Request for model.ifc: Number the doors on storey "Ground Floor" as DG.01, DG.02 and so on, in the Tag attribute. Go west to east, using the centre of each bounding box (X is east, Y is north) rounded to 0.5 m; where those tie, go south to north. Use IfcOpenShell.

First a look at what the model holds.

```python
import ifcopenshell
import ifcopenshell.util.element
import ifcopenshell.util.placement

model = ifcopenshell.open("model.ifc")
print(model.schema)
storey = next(s for s in model.by_type("IfcBuildingStorey") if s.Name == "Ground Floor")
doors = [e for e in ifcopenshell.util.element.get_decomposition(storey) if e.is_a("IfcDoor")]
for e in sorted(doors, key=lambda e: e.id()):
    origin = ifcopenshell.util.placement.get_local_placement(e.ObjectPlacement)[:3, 3]
    print(e.id(), e.Tag, e.Name, origin.round(2) + 0.0, sep=" | ")
```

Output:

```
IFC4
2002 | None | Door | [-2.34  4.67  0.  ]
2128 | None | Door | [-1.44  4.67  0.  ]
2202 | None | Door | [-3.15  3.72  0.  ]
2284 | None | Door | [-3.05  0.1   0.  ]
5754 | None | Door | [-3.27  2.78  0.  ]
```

```python
import ifcopenshell
import ifcopenshell.geom
import ifcopenshell.util.element
import ifcopenshell.util.shape

model = ifcopenshell.open("model.ifc")
settings = ifcopenshell.geom.settings()
settings.set("use-world-coords", True)


def centre(element):
    shape = ifcopenshell.geom.create_shape(settings, element)
    return ifcopenshell.util.shape.get_bbox_centroid(shape.geometry)


storey = next(s for s in model.by_type("IfcBuildingStorey") if s.Name == "Ground Floor")
doors = [e for e in ifcopenshell.util.element.get_decomposition(storey) if e.is_a("IfcDoor")]

# Insertion points can sit at a corner or the storey origin, so sort by the geometry (in metres).
centres = {e: centre(e) for e in doors}
doors.sort(key=lambda e: (round(centres[e][0] / 0.5), centres[e][1]))

for i, e in enumerate(doors, start=1):
    number = f"DG.{i:02d}"
    e.Tag = number
    print(e.id(), number)

model.write("model_rev.ifc")
```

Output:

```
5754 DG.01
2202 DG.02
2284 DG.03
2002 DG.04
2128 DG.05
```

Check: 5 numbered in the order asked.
